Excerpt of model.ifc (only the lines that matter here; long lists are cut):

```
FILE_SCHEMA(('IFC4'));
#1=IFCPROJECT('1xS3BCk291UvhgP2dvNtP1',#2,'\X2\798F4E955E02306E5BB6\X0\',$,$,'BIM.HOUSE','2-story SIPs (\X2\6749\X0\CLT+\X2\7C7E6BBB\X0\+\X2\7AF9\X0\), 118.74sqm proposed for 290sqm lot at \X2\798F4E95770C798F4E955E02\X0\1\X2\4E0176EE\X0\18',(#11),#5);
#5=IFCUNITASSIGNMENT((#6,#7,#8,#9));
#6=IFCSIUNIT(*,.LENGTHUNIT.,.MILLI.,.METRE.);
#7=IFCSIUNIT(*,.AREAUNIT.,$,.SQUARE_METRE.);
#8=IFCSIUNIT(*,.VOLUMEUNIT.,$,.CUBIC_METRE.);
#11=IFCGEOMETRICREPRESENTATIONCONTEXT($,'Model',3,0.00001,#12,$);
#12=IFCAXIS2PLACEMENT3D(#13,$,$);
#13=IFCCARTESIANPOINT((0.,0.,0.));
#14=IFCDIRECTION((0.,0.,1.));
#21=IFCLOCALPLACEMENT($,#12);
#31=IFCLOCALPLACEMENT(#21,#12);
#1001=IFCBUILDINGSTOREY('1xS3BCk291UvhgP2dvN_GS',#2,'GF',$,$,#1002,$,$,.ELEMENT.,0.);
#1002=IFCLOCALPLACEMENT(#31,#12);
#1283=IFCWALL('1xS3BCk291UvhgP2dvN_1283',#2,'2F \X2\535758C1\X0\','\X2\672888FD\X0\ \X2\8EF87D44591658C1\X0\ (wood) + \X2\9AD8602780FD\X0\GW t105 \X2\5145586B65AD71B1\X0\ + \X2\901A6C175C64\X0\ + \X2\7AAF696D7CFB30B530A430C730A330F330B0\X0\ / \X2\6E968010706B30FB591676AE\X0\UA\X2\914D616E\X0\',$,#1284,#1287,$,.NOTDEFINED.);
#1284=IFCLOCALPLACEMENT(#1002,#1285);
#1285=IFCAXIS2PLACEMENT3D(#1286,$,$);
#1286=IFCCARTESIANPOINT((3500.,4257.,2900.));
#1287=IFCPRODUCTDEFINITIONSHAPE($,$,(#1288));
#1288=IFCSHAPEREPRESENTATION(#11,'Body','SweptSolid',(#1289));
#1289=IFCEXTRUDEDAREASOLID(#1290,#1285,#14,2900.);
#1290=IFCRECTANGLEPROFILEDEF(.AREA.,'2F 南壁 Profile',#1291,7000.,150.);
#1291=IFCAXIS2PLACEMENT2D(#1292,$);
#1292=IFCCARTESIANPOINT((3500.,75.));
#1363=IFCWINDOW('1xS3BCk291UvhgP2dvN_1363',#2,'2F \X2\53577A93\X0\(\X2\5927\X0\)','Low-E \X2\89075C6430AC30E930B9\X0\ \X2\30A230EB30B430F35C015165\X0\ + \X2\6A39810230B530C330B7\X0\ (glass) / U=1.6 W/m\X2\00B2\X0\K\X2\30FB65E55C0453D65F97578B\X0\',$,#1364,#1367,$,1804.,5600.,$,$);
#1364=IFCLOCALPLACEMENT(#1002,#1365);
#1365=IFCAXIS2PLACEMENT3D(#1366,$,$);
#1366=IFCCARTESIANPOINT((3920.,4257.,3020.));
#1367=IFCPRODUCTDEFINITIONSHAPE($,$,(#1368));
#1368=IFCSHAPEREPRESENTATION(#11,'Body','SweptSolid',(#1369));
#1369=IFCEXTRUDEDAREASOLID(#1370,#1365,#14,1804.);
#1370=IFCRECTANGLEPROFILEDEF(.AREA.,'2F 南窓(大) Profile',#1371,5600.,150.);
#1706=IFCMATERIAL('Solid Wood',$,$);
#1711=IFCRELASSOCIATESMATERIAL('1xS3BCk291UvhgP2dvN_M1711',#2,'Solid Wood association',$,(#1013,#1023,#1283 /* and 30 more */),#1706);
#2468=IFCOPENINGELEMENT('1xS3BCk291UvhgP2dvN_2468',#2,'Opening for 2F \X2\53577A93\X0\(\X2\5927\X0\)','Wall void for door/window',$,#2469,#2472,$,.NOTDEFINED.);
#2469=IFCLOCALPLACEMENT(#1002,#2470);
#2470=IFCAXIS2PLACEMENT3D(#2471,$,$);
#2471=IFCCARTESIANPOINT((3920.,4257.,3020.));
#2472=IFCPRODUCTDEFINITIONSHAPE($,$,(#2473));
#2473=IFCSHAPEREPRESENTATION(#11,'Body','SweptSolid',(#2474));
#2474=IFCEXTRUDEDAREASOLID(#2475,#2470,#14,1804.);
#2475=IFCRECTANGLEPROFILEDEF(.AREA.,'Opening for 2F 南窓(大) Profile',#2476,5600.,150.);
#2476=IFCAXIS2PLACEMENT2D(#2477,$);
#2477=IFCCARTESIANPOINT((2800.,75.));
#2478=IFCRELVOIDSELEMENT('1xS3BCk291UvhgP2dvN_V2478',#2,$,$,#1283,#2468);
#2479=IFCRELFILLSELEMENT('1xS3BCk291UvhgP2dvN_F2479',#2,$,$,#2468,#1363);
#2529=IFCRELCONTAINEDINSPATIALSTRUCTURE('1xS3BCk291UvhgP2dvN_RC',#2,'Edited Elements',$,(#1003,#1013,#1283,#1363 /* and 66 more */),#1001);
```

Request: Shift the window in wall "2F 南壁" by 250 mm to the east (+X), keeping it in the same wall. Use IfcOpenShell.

```python
import ifcopenshell
import ifcopenshell.api.geometry
import ifcopenshell.util.placement
import ifcopenshell.util.unit

model = ifcopenshell.open("model.ifc")
unit_scale = ifcopenshell.util.unit.calculate_unit_scale(model)

window = model.by_guid("1xS3BCk291UvhgP2dvN_1363")
opening = window.FillsVoids[0].RelatingOpeningElement
wall = opening.VoidsElements[0].RelatingBuildingElement

wall_matrix = ifcopenshell.util.placement.get_local_placement(wall.ObjectPlacement)
shift = wall_matrix[:3, 0] * 0.25 / unit_scale
before = ifcopenshell.util.placement.get_local_placement(window.ObjectPlacement)[:3, 3].copy()

# The window is not placed relative to its opening, so move both.
for product in (opening, window):
    matrix = ifcopenshell.util.placement.get_local_placement(product.ObjectPlacement)
    matrix[:3, 3] += shift
    ifcopenshell.api.geometry.edit_object_placement(model, product=product, matrix=matrix, is_si=False)

after = ifcopenshell.util.placement.get_local_placement(window.ObjectPlacement)[:3, 3]
print("window moved by", (after - before).round(3) + 0.0)

model.write("model_updated.ifc")
```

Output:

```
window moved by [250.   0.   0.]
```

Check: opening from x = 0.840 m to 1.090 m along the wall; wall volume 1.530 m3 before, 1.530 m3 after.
